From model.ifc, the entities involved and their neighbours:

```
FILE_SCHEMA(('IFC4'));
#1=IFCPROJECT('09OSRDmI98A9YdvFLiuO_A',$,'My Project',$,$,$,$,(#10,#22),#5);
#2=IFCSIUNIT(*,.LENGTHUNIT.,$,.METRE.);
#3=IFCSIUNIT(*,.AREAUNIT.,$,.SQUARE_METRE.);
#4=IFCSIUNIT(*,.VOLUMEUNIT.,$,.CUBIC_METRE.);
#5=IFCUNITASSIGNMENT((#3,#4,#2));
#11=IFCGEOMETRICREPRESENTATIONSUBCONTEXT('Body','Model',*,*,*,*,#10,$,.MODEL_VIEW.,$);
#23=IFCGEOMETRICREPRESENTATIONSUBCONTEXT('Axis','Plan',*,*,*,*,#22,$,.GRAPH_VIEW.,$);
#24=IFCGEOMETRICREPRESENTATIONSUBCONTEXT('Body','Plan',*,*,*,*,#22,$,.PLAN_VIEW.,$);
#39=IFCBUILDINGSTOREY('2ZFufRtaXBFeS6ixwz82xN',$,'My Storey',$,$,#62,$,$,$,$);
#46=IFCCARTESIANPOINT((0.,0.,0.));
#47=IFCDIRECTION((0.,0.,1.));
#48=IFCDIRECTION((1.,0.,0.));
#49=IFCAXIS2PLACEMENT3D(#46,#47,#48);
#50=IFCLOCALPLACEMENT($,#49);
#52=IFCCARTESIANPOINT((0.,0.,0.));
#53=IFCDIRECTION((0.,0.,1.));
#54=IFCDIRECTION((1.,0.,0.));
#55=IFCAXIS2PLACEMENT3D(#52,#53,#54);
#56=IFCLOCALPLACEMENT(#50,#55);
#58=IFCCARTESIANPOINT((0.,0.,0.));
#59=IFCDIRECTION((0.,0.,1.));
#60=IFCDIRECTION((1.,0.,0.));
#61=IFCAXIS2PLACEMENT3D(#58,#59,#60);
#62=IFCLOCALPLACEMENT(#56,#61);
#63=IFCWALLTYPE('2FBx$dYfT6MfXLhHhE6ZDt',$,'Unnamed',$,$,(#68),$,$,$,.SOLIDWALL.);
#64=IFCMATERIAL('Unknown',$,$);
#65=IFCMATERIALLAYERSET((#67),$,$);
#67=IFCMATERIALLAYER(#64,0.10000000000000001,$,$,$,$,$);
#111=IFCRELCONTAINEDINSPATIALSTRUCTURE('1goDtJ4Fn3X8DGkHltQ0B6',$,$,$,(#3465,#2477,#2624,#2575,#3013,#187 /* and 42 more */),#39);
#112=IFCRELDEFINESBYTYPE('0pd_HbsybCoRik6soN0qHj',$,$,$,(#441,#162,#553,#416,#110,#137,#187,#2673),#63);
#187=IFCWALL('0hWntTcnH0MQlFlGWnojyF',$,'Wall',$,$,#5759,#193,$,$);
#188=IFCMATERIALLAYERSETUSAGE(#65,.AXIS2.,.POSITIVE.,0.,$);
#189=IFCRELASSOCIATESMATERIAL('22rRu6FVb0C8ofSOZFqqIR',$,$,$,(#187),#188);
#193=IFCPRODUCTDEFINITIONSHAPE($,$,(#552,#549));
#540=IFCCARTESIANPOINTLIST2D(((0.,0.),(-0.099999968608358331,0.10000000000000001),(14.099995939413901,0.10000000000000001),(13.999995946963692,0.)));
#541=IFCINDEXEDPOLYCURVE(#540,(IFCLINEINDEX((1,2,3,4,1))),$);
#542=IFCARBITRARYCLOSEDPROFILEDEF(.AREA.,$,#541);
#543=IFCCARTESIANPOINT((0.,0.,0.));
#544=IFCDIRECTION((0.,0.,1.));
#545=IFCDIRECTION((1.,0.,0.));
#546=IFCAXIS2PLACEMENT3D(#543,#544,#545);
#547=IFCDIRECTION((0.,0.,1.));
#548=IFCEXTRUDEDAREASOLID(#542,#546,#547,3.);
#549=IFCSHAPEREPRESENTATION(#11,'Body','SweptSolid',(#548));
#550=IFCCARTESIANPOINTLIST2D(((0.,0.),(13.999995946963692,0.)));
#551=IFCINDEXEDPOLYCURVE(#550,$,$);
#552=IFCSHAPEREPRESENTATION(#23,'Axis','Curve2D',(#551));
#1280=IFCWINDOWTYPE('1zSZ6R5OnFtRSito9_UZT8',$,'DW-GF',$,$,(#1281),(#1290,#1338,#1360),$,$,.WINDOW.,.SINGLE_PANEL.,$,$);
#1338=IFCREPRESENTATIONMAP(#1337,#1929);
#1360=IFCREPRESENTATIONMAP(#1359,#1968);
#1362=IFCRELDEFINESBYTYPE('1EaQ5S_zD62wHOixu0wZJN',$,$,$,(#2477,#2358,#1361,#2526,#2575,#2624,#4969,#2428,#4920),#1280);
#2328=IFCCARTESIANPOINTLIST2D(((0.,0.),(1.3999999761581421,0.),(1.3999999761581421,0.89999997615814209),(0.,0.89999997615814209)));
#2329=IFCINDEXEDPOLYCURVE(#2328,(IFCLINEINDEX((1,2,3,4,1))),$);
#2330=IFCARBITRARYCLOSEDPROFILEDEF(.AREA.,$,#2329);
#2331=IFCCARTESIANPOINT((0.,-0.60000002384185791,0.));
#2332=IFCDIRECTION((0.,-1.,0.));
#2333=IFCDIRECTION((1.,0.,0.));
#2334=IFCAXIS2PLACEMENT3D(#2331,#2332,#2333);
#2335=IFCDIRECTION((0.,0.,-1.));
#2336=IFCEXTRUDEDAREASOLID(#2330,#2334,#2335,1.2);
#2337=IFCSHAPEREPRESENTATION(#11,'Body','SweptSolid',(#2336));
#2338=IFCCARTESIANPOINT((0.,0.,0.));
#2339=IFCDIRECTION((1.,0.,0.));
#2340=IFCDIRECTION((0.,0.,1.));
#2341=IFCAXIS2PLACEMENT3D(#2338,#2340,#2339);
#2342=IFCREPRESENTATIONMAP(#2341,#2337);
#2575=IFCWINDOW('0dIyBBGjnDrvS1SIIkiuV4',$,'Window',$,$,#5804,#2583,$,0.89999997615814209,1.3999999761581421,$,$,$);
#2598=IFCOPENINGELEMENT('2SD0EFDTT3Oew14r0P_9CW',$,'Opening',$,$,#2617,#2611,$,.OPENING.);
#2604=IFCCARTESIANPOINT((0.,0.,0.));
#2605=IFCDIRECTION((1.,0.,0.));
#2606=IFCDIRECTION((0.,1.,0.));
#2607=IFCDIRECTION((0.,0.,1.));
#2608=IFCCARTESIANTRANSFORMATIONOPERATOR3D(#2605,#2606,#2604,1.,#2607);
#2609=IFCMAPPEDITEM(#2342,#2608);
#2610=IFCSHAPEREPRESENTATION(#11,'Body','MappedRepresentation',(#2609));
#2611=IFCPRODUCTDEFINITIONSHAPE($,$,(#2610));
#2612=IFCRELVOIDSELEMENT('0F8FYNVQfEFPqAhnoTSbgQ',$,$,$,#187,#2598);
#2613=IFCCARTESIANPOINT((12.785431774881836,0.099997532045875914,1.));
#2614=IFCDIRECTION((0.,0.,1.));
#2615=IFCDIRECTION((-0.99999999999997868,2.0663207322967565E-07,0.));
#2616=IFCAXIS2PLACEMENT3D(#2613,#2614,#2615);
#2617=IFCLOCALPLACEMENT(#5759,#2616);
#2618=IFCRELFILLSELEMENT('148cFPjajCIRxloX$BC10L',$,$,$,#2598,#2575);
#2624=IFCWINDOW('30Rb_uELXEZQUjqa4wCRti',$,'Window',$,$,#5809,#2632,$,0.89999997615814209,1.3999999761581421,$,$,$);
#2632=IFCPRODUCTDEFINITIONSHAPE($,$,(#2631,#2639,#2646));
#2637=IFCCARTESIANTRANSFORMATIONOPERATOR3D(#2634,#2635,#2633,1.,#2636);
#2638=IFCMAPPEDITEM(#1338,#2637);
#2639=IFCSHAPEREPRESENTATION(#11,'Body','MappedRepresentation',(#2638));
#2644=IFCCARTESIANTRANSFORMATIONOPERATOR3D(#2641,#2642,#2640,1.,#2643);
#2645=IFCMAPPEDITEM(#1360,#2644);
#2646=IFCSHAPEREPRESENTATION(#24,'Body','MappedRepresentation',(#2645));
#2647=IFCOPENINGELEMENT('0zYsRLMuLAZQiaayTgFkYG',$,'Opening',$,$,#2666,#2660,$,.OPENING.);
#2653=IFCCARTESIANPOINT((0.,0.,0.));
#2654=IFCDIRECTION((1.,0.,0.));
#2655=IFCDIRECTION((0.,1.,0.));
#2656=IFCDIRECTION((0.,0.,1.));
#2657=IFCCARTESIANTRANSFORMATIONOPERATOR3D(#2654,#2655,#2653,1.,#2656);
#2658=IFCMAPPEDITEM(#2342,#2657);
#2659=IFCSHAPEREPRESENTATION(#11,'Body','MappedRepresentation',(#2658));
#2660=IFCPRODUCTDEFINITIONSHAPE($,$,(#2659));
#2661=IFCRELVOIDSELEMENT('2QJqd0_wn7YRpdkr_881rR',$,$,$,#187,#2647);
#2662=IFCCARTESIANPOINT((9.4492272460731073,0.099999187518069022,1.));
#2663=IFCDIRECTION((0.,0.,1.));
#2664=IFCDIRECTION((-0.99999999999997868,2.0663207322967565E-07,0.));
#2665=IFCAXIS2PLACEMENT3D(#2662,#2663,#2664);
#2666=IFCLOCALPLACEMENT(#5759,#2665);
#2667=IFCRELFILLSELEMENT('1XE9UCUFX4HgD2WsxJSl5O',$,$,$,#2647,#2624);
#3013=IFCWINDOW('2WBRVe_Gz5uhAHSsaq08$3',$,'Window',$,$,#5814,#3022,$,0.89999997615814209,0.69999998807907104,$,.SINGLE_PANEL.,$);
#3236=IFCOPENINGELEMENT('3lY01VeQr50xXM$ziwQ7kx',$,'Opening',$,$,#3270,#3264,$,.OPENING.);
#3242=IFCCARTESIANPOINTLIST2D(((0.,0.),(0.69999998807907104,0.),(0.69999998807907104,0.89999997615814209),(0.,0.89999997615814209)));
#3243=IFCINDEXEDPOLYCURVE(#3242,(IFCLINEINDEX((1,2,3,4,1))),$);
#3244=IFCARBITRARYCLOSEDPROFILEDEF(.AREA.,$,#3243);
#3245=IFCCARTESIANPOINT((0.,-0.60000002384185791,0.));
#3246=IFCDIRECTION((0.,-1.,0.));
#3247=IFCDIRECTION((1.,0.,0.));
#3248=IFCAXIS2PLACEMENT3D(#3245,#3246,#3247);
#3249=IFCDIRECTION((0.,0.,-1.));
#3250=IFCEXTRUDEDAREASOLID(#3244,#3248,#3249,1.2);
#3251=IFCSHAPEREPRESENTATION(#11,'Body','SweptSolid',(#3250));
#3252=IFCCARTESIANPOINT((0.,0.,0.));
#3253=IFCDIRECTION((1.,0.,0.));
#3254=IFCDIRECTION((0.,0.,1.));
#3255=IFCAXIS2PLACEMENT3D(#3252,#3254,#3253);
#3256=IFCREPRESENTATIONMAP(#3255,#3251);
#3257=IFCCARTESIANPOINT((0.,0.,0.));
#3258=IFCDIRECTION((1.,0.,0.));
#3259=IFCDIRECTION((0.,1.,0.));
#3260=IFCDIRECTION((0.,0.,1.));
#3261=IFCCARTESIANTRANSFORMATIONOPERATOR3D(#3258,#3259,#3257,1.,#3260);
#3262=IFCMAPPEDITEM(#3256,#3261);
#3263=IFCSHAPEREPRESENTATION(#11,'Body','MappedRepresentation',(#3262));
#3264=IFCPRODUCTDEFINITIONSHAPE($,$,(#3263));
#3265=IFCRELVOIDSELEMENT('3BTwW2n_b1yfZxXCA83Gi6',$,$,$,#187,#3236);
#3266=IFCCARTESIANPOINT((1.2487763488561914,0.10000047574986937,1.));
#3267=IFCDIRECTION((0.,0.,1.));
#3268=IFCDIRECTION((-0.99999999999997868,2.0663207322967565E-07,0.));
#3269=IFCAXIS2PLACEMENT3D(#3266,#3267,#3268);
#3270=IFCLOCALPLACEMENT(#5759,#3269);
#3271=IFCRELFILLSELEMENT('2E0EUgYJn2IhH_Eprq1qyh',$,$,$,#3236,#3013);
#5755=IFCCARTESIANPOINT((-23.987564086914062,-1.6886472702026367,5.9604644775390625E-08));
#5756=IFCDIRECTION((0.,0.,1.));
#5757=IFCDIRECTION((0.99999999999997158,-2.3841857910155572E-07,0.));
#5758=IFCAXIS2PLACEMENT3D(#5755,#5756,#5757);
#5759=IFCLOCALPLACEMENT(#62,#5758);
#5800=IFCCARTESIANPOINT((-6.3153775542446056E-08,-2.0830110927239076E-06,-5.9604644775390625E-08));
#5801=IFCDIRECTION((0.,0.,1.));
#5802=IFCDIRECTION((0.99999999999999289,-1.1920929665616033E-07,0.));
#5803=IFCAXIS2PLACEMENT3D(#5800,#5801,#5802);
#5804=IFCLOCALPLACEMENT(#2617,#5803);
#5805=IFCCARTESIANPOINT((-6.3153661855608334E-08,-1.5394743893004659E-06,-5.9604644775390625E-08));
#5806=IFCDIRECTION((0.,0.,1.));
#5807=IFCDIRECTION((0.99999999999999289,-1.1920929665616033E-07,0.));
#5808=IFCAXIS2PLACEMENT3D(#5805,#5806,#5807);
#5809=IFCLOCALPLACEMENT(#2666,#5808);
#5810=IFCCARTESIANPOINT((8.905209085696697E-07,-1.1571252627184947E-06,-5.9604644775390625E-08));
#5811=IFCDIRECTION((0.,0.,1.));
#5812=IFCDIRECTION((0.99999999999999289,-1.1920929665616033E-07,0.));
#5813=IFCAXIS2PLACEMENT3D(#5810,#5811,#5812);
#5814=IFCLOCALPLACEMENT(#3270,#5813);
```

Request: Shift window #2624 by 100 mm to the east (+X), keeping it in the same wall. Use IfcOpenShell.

```python
import ifcopenshell
import ifcopenshell.api.geometry
import ifcopenshell.util.placement

model = ifcopenshell.open("model.ifc")

window = model.by_guid("30Rb_uELXEZQUjqa4wCRti")
opening = window.FillsVoids[0].RelatingOpeningElement
wall = opening.VoidsElements[0].RelatingBuildingElement

wall_matrix = ifcopenshell.util.placement.get_local_placement(wall.ObjectPlacement)
shift = wall_matrix[:3, 0] * 0.1
before = ifcopenshell.util.placement.get_local_placement(window.ObjectPlacement)[:3, 3].copy()

# The window is placed relative to its opening, so it follows when the opening moves.
matrix = ifcopenshell.util.placement.get_local_placement(opening.ObjectPlacement)
matrix[:3, 3] += shift
ifcopenshell.api.geometry.edit_object_placement(
    model, product=opening, matrix=matrix, is_si=False, should_transform_children=True
)

after = ifcopenshell.util.placement.get_local_placement(window.ObjectPlacement)[:3, 3]
print("window moved by", (after - before).round(3) + 0.0)

model.write("model_updated.ifc")
```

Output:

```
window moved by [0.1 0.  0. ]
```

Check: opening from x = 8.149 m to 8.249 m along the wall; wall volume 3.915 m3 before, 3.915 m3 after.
